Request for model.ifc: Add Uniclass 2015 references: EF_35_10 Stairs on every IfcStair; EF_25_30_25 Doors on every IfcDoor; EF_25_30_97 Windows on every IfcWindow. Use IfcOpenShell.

First a look at what the model holds.

```python
import ifcopenshell

model = ifcopenshell.open("model.ifc")
print(model.schema)
print("classifications:", [c.Name for c in model.by_type("IfcClassification")])
for ifc_class in ("IfcDoor", "IfcRoof", "IfcStair", "IfcWall", "IfcWindow"):
    print(ifc_class, len(model.by_type(ifc_class)))
```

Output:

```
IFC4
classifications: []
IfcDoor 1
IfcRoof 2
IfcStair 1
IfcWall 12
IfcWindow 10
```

```python
import ifcopenshell
import ifcopenshell.api.classification

model = ifcopenshell.open("model.ifc")

system = ifcopenshell.api.classification.add_classification(model, classification="Uniclass 2015")

codes = {
    "IfcStair": ("EF_35_10", "Stairs"),
    "IfcDoor": ("EF_25_30_25", "Doors"),
    "IfcWindow": ("EF_25_30_97", "Windows"),
}
for ifc_class, (code, name) in codes.items():
    products = model.by_type(ifc_class)
    ifcopenshell.api.classification.add_reference(
        model, products=products, classification=system, identification=code, name=name
    )
    print(code, len(products))

model.write("model-out.ifc")
```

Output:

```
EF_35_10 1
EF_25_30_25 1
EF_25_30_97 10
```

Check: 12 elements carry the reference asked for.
